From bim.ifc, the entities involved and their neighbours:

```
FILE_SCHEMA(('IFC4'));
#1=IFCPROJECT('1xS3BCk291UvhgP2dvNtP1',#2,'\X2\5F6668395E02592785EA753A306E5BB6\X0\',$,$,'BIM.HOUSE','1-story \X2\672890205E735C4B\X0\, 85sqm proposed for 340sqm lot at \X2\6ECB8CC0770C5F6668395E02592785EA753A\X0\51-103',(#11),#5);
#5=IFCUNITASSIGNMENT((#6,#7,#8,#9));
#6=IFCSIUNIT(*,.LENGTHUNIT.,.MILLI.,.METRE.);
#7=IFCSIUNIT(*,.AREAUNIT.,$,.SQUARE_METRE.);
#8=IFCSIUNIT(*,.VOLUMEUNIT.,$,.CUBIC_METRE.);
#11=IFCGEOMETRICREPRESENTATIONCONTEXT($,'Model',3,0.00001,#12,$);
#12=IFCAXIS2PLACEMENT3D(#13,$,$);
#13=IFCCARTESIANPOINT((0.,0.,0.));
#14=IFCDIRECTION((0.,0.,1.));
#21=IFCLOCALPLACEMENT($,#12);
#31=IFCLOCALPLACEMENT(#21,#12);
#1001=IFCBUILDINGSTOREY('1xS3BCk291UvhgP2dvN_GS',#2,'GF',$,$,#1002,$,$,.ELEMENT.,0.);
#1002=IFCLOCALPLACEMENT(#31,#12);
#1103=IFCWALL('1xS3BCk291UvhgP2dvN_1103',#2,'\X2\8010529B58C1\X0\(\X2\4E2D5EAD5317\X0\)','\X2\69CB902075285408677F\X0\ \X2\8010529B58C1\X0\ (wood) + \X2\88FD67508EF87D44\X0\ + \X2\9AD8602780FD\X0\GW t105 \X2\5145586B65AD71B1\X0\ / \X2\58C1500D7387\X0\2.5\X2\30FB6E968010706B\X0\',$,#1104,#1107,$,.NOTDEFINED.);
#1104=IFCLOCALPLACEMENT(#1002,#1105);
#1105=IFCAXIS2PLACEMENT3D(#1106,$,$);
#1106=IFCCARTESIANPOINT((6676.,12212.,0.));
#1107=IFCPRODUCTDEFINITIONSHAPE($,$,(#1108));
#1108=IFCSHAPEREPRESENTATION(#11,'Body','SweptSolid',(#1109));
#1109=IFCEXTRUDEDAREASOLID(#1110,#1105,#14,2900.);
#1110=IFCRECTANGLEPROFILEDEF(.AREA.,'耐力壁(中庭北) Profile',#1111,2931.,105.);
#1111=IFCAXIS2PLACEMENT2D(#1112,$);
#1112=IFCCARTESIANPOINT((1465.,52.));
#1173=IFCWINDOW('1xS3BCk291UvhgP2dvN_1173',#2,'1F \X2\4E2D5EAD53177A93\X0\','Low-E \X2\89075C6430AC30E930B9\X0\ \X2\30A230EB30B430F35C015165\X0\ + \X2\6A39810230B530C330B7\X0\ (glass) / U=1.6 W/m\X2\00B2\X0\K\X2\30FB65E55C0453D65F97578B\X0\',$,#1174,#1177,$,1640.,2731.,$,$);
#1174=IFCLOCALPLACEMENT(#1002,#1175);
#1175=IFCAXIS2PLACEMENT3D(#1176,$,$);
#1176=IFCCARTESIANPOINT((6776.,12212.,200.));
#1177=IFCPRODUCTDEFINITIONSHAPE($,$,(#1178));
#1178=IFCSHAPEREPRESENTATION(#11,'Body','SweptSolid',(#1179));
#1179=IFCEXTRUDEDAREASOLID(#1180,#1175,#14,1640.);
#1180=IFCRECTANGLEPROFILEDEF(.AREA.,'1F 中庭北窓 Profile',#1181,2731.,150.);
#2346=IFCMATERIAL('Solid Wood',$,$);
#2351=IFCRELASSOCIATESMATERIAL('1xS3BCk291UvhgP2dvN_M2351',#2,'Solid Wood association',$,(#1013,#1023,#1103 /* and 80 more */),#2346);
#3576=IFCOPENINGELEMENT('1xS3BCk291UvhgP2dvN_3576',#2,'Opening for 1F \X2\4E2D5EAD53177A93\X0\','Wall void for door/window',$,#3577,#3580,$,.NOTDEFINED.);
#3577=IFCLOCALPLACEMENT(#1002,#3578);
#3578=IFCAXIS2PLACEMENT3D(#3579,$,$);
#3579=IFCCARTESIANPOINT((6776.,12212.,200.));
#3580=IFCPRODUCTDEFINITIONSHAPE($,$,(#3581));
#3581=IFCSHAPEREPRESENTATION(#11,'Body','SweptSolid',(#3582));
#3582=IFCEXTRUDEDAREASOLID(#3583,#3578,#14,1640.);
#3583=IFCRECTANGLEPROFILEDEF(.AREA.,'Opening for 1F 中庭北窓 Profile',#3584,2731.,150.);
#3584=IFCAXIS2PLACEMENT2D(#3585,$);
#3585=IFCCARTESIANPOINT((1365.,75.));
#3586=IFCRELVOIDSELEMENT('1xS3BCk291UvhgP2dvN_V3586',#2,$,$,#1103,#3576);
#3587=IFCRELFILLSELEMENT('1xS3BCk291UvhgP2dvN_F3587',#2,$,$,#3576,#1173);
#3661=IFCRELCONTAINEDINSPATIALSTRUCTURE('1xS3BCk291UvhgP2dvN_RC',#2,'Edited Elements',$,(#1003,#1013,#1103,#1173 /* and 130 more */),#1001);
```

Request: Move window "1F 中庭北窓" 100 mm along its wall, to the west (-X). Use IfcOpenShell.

```python
import ifcopenshell
import ifcopenshell.api.geometry
import ifcopenshell.util.placement
import ifcopenshell.util.unit

model = ifcopenshell.open("bim.ifc")
unit_scale = ifcopenshell.util.unit.calculate_unit_scale(model)

window = model.by_guid("1xS3BCk291UvhgP2dvN_1173")
opening = window.FillsVoids[0].RelatingOpeningElement
wall = opening.VoidsElements[0].RelatingBuildingElement

wall_matrix = ifcopenshell.util.placement.get_local_placement(wall.ObjectPlacement)
shift = wall_matrix[:3, 0] * -0.1 / unit_scale
before = ifcopenshell.util.placement.get_local_placement(window.ObjectPlacement)[:3, 3].copy()

# The window is not placed relative to its opening, so move both.
for product in (opening, window):
    matrix = ifcopenshell.util.placement.get_local_placement(product.ObjectPlacement)
    matrix[:3, 3] += shift
    ifcopenshell.api.geometry.edit_object_placement(model, product=product, matrix=matrix, is_si=False)

after = ifcopenshell.util.placement.get_local_placement(window.ObjectPlacement)[:3, 3]
print("window moved by", (after - before).round(3) + 0.0)

model.write("bim_rev.ifc")
```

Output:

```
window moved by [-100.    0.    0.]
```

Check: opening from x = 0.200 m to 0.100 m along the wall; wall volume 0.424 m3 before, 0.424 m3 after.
